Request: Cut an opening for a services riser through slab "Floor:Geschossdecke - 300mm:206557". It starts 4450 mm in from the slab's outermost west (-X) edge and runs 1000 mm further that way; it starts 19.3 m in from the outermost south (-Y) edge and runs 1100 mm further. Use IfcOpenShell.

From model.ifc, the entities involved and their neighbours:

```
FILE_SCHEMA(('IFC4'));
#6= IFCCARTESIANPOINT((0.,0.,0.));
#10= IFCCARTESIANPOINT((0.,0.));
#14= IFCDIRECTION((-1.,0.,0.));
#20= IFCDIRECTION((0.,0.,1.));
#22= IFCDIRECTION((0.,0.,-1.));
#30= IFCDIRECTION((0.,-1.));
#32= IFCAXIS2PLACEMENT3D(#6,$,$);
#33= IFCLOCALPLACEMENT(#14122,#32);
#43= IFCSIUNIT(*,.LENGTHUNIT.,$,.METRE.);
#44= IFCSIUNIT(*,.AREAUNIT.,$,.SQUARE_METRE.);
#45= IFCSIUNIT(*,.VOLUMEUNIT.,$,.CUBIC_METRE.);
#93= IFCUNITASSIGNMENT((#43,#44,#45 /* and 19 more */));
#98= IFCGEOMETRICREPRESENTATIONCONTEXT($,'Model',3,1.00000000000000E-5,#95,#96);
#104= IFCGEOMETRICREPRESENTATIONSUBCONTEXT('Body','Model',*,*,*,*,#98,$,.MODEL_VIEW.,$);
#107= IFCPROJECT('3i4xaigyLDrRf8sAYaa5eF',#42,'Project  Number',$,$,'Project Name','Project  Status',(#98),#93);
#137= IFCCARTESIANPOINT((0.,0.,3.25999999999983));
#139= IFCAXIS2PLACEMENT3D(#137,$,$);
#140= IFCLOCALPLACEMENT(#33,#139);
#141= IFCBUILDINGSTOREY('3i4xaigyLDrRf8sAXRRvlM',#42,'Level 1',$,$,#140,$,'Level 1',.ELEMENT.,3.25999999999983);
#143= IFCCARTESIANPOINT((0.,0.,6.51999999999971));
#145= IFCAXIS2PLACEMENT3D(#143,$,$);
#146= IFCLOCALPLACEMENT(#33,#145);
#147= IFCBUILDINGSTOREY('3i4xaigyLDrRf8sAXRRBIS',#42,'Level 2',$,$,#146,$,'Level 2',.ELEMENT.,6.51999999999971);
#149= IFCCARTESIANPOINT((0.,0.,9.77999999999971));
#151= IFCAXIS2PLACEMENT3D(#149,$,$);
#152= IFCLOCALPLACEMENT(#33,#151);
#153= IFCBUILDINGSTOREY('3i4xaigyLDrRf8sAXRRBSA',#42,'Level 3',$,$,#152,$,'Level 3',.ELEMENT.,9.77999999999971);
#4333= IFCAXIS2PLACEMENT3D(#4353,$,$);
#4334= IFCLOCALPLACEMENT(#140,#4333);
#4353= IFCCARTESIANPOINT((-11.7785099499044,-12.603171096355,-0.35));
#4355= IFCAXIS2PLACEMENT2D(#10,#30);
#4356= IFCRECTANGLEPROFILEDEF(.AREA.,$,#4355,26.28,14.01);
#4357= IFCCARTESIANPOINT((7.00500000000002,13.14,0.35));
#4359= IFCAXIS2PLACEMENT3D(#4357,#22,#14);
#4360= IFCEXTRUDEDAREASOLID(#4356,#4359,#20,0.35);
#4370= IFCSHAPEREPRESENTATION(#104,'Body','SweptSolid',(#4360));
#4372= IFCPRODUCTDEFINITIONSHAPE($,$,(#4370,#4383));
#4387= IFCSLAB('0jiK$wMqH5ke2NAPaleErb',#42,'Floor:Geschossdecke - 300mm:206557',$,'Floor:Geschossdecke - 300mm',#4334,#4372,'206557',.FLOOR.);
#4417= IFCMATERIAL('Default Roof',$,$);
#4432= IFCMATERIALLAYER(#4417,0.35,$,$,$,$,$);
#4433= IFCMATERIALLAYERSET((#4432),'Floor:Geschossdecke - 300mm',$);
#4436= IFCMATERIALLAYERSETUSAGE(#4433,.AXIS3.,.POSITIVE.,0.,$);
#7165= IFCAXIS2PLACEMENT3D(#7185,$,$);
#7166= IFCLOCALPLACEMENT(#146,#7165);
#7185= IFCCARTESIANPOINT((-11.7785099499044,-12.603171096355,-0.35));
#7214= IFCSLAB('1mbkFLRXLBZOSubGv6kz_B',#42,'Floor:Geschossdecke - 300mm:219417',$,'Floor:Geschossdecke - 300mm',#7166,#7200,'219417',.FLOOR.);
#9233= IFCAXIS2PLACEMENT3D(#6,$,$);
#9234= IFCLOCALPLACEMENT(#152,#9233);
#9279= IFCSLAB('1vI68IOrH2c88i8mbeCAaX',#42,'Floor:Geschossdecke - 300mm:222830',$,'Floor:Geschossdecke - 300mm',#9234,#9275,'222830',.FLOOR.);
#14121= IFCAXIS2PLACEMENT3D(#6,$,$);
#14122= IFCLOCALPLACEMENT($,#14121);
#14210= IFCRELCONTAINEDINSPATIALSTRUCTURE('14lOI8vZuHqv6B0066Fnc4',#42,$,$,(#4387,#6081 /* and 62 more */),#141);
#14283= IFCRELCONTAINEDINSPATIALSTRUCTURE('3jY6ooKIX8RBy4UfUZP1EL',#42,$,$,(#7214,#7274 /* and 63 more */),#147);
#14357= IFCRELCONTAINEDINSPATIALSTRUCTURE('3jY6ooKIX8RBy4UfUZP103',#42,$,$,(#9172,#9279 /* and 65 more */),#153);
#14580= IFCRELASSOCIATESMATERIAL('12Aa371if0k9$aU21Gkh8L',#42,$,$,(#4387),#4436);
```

```python
import numpy as np
import ifcopenshell
import ifcopenshell.api.feature
import ifcopenshell.api.geometry
import ifcopenshell.api.root
import ifcopenshell.geom
import ifcopenshell.util.placement
import ifcopenshell.util.representation
import ifcopenshell.util.shape
import ifcopenshell.util.unit

model = ifcopenshell.open("model.ifc")
unit_scale = ifcopenshell.util.unit.calculate_unit_scale(model)
settings = ifcopenshell.geom.settings()


def volume(element):
    """Net volume in cubic metres, openings subtracted."""
    shape = ifcopenshell.geom.create_shape(settings, element)
    return ifcopenshell.util.shape.get_volume(shape.geometry)


slab = model.by_guid("0jiK$wMqH5ke2NAPaleErb")
before = volume(slab)

# Extent in the slab's own axes, in metres. The edges named are its -X and -Y sides.
slab_shape = ifcopenshell.geom.create_shape(settings, slab)
vertices = ifcopenshell.util.shape.get_vertices(slab_shape.geometry)
x_min, y_min, bottom = vertices.min(axis=0)
top = vertices[:, 2].max()

opening = ifcopenshell.api.root.create_entity(model, ifc_class="IfcOpeningElement", name="Services riser opening", predefined_type="OPENING")
context = ifcopenshell.util.representation.get_context(model, "Model", "Body", "MODEL_VIEW")
width, depth = 1, 1.1
outline = [(0.0, 0.0), (width, 0.0), (width, depth), (0.0, depth), (0.0, 0.0)]
# Overshoot both faces by 50 mm so the cut is clean.
shape = ifcopenshell.api.geometry.add_slab_representation(
    model, context=context, depth=top - bottom + 0.1, polyline=outline
)
ifcopenshell.api.geometry.assign_representation(model, product=opening, representation=shape)

matrix = ifcopenshell.util.placement.get_local_placement(slab.ObjectPlacement)
matrix[:, 3] = matrix @ np.append(np.array([x_min + 4.45, y_min + 19.3, bottom - 0.05]) / unit_scale, 1.0)
ifcopenshell.api.geometry.edit_object_placement(model, product=opening, matrix=matrix, is_si=False)
ifcopenshell.api.feature.add_feature(model, feature=opening, element=slab)

after = volume(slab)

print(f"slab volume {before:.3f} -> {after:.3f} m3")

model.write("model_updated.ifc")
```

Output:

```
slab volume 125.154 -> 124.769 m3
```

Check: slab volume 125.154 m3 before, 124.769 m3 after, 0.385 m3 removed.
